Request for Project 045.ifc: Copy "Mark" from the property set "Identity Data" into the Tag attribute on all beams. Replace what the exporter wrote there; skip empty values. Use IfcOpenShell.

First a look at what the model holds.

```python
import ifcopenshell
import ifcopenshell.util.element

model = ifcopenshell.open("Project 045.ifc")
print(model.schema)
beams = model.by_type("IfcBeam")
print(len(beams), "beams")
for e in beams[:8]:
    source = ifcopenshell.util.element.get_pset(e, "Identity Data", "Mark")
    target = e.Tag
    print(e.id(), repr(source), repr(target), sep=" | ")
```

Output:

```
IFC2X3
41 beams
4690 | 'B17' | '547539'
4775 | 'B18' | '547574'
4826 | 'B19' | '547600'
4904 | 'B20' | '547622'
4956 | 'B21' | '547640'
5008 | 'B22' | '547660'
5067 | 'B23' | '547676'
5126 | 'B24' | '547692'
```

```python
import ifcopenshell
import ifcopenshell.util.element

model = ifcopenshell.open("Project 045.ifc")

count = 0
for e in model.by_type("IfcBeam"):
    value = ifcopenshell.util.element.get_pset(e, "Identity Data", "Mark")
    current = e.Tag
    if not value or not value.strip() or current == value:
        continue
    e.Tag = value
    count += 1

print(count, "beams updated")

model.write("Project 045-out.ifc")
```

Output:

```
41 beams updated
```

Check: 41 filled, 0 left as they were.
